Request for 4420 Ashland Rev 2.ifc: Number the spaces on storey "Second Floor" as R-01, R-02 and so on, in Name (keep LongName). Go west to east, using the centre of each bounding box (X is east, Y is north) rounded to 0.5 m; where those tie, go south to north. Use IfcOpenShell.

First a look at what the model holds.

```python
import ifcopenshell
import ifcopenshell.util.element
import ifcopenshell.util.placement

model = ifcopenshell.open("4420 Ashland Rev 2.ifc")
print(model.schema)
storey = next(s for s in model.by_type("IfcBuildingStorey") if s.Name == "Second Floor")
spaces = [e for e in ifcopenshell.util.element.get_decomposition(storey) if e.is_a("IfcSpace")]
for e in sorted(spaces, key=lambda e: e.id()):
    origin = ifcopenshell.util.placement.get_local_placement(e.ObjectPlacement)[:3, 3]
    print(e.id(), e.Name, e.LongName, origin.round(2) + 0.0, sep=" | ")
```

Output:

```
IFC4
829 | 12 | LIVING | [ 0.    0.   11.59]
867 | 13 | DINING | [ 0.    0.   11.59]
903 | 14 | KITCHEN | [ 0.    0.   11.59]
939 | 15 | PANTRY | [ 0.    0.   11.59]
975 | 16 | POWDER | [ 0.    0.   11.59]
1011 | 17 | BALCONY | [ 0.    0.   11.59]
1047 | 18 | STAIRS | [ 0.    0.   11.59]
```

```python
import ifcopenshell
import ifcopenshell.geom
import ifcopenshell.util.element
import ifcopenshell.util.shape

model = ifcopenshell.open("4420 Ashland Rev 2.ifc")
settings = ifcopenshell.geom.settings()
settings.set("use-world-coords", True)


def centre(element):
    shape = ifcopenshell.geom.create_shape(settings, element)
    return ifcopenshell.util.shape.get_bbox_centroid(shape.geometry)


storey = next(s for s in model.by_type("IfcBuildingStorey") if s.Name == "Second Floor")
spaces = [e for e in ifcopenshell.util.element.get_decomposition(storey) if e.is_a("IfcSpace")]

# Insertion points can sit at a corner or the storey origin, so sort by the geometry (in metres).
centres = {e: centre(e) for e in spaces}
spaces.sort(key=lambda e: (round(centres[e][0] / 0.5), centres[e][1]))

for i, e in enumerate(spaces, start=1):
    number = f"R-{i:02d}"
    e.Name = number
    print(e.id(), number)

model.write("4420 Ashland Rev 2_v2.ifc")
```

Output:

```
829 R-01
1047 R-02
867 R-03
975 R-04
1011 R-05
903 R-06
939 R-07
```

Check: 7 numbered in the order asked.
